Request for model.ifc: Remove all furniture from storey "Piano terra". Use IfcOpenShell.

First a look at what the model holds.

```python
import ifcopenshell
import ifcopenshell.util.element

model = ifcopenshell.open("model.ifc")
print(model.schema)
storey = next(s for s in model.by_type("IfcBuildingStorey") if s.Name == "Piano terra")
furniture = [e for e in ifcopenshell.util.element.get_decomposition(storey) if e.is_a("IfcFurnishingElement")]
seen = {}
for e in furniture:
    element_type = ifcopenshell.util.element.get_type(e)
    name = element_type.Name if element_type not in (None, e) else None
    seen[name] = seen.get(name, 0) + 1
for name, count in sorted(seen.items(), key=str):
    print(count, "x", name)
```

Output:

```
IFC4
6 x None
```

```python
import ifcopenshell
import ifcopenshell.api.root
import ifcopenshell.util.element

model = ifcopenshell.open("model.ifc")

storey = next(s for s in model.by_type("IfcBuildingStorey") if s.Name == "Piano terra")
furniture = [e for e in ifcopenshell.util.element.get_decomposition(storey) if e.is_a("IfcFurnishingElement")]

for e in furniture:
    ifcopenshell.api.root.remove_product(model, product=e)
print(len(furniture), "removed")

model.write("model_v2.ifc")
```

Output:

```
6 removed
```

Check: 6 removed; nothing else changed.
